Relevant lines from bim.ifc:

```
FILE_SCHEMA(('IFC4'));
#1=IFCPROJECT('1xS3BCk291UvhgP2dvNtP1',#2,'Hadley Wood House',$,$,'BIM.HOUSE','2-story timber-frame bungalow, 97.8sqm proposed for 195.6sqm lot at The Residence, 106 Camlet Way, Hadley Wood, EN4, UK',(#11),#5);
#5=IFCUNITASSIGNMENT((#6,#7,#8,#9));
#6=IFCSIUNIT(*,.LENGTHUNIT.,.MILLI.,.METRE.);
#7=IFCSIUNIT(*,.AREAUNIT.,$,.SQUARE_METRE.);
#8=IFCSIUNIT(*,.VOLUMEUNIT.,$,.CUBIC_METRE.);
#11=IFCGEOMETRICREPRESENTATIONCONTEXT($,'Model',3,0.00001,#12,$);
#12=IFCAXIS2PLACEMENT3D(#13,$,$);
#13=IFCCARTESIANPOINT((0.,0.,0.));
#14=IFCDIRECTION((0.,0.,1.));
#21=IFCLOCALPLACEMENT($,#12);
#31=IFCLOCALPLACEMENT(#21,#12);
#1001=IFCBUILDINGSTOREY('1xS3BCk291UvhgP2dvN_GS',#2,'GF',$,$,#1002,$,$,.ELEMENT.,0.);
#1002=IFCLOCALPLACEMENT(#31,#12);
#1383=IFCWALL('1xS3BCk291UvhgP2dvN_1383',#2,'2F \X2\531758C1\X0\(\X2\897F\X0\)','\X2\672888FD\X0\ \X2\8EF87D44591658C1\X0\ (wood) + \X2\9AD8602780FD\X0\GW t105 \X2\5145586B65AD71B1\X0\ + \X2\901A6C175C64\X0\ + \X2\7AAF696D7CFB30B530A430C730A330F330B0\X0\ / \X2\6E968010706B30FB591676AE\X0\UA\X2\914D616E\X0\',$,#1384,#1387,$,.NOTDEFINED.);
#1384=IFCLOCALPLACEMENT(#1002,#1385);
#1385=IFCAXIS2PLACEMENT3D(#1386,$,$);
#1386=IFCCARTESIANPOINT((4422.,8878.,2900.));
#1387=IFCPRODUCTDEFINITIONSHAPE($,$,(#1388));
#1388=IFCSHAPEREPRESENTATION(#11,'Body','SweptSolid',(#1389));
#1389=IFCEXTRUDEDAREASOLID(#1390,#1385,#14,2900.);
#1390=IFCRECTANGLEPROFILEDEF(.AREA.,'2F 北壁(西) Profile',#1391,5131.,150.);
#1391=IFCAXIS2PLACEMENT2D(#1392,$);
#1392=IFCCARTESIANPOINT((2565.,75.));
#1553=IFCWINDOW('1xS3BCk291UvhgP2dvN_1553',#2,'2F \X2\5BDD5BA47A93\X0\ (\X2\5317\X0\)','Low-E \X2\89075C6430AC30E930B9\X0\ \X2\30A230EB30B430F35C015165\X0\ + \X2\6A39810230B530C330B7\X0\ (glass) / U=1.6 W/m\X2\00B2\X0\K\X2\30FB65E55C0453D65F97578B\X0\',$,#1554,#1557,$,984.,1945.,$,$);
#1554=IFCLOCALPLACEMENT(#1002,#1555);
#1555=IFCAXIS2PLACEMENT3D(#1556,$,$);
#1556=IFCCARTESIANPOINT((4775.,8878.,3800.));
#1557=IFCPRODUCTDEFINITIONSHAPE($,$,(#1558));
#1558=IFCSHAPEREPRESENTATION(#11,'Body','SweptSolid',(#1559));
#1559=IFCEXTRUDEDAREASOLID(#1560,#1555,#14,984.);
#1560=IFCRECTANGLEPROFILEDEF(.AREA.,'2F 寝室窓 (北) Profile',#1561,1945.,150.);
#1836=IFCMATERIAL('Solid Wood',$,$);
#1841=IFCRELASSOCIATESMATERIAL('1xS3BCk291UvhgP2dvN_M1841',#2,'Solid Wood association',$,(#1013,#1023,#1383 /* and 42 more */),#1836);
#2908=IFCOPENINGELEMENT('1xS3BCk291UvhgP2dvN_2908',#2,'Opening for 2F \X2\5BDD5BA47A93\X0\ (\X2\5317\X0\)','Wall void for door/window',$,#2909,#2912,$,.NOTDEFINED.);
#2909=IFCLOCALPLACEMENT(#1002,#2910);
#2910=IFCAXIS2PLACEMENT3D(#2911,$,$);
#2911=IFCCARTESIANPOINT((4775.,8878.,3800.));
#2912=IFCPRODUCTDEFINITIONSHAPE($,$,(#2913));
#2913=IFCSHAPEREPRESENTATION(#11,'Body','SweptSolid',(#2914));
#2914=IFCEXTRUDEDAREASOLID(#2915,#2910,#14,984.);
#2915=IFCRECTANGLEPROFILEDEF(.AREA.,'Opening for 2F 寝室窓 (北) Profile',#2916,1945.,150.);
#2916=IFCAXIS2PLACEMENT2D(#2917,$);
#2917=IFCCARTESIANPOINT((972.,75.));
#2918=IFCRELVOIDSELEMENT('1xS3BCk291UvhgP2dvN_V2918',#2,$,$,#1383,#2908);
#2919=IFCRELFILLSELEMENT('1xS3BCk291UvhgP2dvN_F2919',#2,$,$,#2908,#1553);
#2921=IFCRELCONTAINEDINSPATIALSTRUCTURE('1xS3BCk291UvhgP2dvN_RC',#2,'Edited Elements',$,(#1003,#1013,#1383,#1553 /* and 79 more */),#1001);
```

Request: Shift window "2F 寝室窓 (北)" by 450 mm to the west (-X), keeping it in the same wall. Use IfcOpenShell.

```python
import ifcopenshell
import ifcopenshell.api.geometry
import ifcopenshell.util.placement
import ifcopenshell.util.unit

model = ifcopenshell.open("bim.ifc")
unit_scale = ifcopenshell.util.unit.calculate_unit_scale(model)

window = model.by_guid("1xS3BCk291UvhgP2dvN_1553")
opening = window.FillsVoids[0].RelatingOpeningElement
wall = opening.VoidsElements[0].RelatingBuildingElement

wall_matrix = ifcopenshell.util.placement.get_local_placement(wall.ObjectPlacement)
shift = wall_matrix[:3, 0] * -0.45 / unit_scale
before = ifcopenshell.util.placement.get_local_placement(window.ObjectPlacement)[:3, 3].copy()

# The window is not placed relative to its opening, so move both.
for product in (opening, window):
    matrix = ifcopenshell.util.placement.get_local_placement(product.ObjectPlacement)
    matrix[:3, 3] += shift
    ifcopenshell.api.geometry.edit_object_placement(model, product=product, matrix=matrix, is_si=False)

after = ifcopenshell.util.placement.get_local_placement(window.ObjectPlacement)[:3, 3]
print("window moved by", (after - before).round(3) + 0.0)

model.write("bim_rev.ifc")
```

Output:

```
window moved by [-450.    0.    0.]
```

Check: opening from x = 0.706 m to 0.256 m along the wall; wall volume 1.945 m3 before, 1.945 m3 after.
